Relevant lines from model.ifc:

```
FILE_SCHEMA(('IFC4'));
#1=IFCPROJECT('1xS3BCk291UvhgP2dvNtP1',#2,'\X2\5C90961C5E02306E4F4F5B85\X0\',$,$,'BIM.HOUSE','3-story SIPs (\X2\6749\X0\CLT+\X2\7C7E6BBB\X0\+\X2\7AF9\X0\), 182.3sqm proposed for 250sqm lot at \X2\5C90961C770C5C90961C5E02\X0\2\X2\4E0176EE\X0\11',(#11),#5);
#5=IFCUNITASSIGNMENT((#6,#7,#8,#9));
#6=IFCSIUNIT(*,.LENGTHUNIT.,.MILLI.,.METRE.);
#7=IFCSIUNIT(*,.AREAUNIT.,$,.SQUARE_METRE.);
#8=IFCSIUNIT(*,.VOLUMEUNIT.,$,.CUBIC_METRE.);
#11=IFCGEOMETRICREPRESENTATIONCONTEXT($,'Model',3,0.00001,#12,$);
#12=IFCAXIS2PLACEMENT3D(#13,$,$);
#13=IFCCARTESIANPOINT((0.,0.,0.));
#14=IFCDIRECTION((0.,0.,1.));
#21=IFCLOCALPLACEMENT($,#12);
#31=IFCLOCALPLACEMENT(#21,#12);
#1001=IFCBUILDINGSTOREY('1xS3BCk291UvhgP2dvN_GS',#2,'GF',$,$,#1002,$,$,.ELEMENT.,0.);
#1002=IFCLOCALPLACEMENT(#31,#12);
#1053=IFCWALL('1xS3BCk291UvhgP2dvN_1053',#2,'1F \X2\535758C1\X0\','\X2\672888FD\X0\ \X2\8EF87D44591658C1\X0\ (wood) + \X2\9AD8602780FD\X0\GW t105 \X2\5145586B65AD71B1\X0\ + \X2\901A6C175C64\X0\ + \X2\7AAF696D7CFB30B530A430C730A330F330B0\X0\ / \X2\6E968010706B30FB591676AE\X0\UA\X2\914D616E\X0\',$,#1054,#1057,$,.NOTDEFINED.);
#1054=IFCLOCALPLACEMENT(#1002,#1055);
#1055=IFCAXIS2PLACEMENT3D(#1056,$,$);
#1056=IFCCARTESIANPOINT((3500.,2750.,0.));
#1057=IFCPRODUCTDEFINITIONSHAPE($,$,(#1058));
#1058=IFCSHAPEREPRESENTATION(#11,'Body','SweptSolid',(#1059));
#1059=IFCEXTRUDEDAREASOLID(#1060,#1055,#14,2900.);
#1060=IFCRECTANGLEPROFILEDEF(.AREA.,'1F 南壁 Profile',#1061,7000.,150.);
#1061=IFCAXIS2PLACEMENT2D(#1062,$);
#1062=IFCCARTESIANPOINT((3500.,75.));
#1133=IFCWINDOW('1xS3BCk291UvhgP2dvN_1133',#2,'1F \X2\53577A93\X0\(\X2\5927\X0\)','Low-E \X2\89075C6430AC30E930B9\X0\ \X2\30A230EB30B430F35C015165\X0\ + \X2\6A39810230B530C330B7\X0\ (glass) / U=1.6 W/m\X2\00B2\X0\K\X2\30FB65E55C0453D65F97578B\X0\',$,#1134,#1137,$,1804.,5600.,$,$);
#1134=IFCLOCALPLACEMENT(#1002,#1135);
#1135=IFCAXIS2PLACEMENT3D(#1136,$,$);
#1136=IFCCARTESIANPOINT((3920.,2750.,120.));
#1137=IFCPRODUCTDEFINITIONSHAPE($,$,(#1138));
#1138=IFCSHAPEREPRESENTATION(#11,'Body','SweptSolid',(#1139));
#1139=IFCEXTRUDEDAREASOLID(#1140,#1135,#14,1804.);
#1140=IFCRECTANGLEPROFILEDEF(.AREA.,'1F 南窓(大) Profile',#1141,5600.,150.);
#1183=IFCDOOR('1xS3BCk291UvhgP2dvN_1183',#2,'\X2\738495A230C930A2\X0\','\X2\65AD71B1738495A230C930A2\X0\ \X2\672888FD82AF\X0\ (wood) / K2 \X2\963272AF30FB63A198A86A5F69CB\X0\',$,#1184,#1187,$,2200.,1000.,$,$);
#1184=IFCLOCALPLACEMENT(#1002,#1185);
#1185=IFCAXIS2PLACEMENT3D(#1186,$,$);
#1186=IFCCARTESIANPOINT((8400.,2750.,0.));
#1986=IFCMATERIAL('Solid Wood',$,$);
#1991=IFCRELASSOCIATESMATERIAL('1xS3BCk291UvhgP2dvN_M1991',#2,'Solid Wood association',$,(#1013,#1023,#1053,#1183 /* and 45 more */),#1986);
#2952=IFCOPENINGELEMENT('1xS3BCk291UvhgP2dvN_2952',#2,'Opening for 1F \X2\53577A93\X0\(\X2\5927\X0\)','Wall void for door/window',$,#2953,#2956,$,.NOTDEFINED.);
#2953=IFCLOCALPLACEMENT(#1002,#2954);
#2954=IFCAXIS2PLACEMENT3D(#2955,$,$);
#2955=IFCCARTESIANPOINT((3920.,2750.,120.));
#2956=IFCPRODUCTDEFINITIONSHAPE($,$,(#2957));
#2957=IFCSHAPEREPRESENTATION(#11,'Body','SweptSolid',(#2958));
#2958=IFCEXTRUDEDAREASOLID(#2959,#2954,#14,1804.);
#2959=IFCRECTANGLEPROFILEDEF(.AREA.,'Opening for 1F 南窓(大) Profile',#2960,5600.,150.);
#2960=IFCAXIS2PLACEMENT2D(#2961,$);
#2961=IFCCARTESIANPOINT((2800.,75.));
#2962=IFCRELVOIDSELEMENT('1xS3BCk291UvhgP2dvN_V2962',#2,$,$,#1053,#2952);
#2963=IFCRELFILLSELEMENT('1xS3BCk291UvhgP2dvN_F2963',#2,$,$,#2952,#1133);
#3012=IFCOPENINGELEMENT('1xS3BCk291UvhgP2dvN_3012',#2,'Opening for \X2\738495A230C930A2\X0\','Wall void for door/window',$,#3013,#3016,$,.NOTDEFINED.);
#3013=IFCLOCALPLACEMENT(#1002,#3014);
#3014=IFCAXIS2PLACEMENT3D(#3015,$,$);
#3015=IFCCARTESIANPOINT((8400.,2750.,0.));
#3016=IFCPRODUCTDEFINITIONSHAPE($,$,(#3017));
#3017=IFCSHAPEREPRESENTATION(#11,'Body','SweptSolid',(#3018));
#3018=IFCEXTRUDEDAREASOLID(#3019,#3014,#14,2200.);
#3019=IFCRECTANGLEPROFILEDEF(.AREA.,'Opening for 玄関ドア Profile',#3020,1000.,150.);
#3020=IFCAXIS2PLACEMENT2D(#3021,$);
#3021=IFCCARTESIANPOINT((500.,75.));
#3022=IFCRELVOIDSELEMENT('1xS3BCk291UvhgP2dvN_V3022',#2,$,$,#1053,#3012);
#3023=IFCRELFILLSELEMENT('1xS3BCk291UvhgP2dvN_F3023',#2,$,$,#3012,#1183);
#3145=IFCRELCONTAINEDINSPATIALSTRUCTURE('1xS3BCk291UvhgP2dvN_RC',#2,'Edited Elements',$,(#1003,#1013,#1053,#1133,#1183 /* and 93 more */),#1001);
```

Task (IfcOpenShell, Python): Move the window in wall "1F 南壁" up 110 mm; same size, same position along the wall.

```python
import numpy as np
import ifcopenshell
import ifcopenshell.api.geometry
import ifcopenshell.util.placement
import ifcopenshell.util.unit

model = ifcopenshell.open("model.ifc")
unit_scale = ifcopenshell.util.unit.calculate_unit_scale(model)

window = model.by_id(1133)
opening = window.FillsVoids[0].RelatingOpeningElement
dz = 110.0

shift = np.array([0.0, 0.0, dz])
# The window is not placed relative to its opening, so move both.
for product in (opening, window):
    matrix = ifcopenshell.util.placement.get_local_placement(product.ObjectPlacement)
    matrix[:3, 3] += shift
    ifcopenshell.api.geometry.edit_object_placement(model, product=product, matrix=matrix, is_si=False)

print(f"moved by {dz * unit_scale:+.3f} m")

model.write("model-out.ifc")
```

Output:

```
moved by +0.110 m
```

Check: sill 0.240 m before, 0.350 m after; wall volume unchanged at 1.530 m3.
